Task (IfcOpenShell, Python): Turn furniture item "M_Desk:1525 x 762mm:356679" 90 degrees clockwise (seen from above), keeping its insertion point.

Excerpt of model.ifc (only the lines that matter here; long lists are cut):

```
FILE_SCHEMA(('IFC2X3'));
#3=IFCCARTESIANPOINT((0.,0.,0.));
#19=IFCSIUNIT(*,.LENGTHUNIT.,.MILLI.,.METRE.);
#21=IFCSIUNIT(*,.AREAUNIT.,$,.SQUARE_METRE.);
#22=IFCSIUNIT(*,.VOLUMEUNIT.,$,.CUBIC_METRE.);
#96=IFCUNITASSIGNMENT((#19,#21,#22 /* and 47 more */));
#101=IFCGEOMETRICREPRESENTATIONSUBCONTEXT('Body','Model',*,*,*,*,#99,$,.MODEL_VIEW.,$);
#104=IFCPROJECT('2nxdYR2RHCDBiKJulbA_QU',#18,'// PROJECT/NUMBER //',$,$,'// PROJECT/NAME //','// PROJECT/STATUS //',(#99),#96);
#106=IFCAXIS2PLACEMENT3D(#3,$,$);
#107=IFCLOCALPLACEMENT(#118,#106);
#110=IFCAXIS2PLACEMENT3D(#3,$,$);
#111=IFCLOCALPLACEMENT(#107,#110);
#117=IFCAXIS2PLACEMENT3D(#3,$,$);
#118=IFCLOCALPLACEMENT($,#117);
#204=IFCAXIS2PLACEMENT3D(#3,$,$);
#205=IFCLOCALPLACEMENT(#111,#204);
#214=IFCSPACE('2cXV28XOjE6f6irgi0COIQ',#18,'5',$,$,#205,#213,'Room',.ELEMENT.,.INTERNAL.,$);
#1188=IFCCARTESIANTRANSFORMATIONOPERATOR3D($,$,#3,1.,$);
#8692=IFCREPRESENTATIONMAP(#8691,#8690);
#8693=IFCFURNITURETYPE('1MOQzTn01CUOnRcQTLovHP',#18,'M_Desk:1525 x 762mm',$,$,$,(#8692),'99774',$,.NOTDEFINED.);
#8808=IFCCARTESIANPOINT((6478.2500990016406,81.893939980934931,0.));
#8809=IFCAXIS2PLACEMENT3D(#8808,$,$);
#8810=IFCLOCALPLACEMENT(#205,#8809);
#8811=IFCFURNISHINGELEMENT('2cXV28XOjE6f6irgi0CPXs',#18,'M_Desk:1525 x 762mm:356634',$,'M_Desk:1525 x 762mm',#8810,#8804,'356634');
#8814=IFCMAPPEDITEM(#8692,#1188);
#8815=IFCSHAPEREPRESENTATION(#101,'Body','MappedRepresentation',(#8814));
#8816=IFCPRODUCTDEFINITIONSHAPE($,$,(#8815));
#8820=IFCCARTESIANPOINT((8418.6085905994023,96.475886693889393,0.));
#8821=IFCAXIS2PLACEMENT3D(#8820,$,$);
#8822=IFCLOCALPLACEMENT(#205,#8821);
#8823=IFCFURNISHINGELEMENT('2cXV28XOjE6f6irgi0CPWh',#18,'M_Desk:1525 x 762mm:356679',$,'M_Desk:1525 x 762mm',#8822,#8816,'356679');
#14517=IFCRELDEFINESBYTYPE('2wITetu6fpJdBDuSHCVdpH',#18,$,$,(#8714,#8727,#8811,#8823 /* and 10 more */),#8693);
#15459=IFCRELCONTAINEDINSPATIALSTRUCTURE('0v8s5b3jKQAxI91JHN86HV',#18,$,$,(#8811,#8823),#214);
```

```python
import ifcopenshell
import ifcopenshell.api.geometry
import ifcopenshell.util.placement

model = ifcopenshell.open("model.ifc")

item = model.by_id(8823)
matrix = ifcopenshell.util.placement.get_local_placement(item.ObjectPlacement)
matrix = matrix @ ifcopenshell.util.placement.rotation(-90, "Z")
ifcopenshell.api.geometry.edit_object_placement(model, product=item, matrix=matrix, is_si=False)

print(ifcopenshell.util.placement.get_local_placement(item.ObjectPlacement).round(3) + 0.0)

model.write("model-out.ifc")
```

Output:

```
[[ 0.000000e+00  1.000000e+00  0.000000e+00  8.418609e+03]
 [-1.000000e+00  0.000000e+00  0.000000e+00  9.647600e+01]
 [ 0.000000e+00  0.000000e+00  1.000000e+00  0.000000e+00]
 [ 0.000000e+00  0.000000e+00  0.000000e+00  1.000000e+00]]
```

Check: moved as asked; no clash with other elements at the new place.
